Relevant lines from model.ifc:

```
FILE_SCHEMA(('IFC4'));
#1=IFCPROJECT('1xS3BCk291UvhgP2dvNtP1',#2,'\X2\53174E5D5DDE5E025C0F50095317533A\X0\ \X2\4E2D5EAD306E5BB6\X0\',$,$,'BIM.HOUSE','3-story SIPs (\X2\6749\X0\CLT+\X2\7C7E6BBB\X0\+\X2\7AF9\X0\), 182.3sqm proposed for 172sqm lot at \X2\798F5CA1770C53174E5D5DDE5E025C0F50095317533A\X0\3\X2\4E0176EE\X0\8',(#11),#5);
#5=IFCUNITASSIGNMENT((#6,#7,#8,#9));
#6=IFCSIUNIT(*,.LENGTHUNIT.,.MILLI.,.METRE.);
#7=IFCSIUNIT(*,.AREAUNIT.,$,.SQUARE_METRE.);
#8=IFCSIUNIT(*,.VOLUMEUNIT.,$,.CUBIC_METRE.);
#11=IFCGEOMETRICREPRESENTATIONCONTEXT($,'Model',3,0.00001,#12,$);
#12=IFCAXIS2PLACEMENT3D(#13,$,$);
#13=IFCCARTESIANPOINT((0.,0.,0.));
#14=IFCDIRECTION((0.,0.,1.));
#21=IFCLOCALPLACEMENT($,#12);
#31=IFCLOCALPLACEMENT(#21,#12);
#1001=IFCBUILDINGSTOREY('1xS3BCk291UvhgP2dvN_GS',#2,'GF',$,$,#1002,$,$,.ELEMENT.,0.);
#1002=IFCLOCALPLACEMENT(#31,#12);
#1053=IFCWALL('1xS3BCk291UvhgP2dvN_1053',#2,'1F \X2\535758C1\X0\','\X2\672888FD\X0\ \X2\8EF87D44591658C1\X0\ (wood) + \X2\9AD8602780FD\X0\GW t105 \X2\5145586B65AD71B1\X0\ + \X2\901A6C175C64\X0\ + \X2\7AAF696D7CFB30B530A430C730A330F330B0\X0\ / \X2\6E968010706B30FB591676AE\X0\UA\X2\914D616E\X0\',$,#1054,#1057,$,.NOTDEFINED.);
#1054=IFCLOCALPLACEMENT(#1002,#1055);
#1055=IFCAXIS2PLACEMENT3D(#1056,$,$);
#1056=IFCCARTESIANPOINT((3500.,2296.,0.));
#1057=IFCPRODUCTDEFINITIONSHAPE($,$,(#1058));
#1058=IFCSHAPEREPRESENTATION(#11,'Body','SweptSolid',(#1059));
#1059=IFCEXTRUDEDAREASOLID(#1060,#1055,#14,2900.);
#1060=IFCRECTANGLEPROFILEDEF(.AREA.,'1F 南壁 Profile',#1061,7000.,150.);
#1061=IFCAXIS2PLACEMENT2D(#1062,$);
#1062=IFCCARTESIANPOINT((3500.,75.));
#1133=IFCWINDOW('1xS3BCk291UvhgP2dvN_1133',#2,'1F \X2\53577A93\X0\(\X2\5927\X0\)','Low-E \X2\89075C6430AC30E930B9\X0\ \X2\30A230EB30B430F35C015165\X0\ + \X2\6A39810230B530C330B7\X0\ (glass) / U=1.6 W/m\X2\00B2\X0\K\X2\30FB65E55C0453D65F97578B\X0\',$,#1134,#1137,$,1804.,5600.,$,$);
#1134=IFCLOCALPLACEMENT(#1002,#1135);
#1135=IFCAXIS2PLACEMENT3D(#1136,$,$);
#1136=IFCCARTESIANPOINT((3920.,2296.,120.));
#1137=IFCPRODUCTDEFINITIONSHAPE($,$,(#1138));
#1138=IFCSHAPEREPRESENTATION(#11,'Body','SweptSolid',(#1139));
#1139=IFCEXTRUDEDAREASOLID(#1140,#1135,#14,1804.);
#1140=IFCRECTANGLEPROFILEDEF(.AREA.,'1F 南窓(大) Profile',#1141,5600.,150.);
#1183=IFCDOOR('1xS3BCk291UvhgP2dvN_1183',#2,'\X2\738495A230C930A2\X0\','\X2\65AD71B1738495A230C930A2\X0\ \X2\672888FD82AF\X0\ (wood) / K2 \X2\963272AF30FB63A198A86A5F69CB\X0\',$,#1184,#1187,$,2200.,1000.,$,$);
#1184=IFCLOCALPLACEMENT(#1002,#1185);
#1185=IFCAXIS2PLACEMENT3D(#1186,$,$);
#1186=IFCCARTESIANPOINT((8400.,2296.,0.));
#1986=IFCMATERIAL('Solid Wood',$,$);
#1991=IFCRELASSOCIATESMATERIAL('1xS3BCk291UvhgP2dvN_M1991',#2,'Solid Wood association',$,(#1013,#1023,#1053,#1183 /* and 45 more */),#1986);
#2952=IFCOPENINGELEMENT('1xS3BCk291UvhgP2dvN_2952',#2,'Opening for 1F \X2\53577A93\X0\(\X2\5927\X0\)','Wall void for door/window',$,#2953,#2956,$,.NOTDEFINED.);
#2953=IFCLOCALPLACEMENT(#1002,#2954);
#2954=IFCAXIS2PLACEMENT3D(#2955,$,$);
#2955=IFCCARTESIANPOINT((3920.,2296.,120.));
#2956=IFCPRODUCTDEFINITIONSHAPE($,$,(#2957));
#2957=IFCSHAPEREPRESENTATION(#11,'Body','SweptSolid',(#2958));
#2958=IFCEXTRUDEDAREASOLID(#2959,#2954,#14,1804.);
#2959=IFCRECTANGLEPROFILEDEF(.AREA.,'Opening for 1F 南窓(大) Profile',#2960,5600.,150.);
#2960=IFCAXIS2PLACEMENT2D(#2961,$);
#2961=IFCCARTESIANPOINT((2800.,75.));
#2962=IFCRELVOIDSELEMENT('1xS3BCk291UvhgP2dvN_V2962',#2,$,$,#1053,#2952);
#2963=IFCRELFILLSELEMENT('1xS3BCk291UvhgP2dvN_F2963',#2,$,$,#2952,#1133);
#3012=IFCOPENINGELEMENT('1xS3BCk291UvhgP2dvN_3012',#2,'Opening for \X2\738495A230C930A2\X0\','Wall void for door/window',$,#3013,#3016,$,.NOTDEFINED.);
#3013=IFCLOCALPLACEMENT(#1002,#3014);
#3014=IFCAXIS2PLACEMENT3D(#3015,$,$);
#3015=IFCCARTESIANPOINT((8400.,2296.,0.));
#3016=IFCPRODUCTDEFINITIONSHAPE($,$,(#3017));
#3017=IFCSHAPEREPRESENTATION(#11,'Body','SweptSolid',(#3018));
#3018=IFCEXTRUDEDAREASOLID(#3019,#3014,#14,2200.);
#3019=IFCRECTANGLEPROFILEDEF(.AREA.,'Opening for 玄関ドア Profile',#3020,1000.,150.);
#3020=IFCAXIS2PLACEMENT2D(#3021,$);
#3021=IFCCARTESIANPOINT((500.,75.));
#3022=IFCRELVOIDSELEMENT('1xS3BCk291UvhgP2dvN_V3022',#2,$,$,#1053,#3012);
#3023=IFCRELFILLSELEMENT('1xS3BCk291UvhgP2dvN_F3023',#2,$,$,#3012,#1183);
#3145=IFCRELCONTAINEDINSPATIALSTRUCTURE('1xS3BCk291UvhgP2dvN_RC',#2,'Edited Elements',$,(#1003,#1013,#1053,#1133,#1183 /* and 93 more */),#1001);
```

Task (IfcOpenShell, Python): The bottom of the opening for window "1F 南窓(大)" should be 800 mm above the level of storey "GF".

```python
import numpy as np
import ifcopenshell
import ifcopenshell.api.geometry
import ifcopenshell.geom
import ifcopenshell.util.element
import ifcopenshell.util.placement
import ifcopenshell.util.shape
import ifcopenshell.util.unit

model = ifcopenshell.open("model.ifc")
unit_scale = ifcopenshell.util.unit.calculate_unit_scale(model)

window = model.by_guid("1xS3BCk291UvhgP2dvN_1133")
opening = window.FillsVoids[0].RelatingOpeningElement
storey = ifcopenshell.util.element.get_container(window, ifc_class="IfcBuildingStorey")
level = ifcopenshell.util.placement.get_local_placement(storey.ObjectPlacement)[2, 3]

# The opening's origin need not be at the sill, so measure its lowest point.
shape = ifcopenshell.geom.create_shape(ifcopenshell.geom.settings(), opening)
bottom = ifcopenshell.util.shape.get_shape_bottom_elevation(shape, shape.geometry) / unit_scale
dz = level + 0.8 / unit_scale - bottom

shift = np.array([0.0, 0.0, dz])
# The window is not placed relative to its opening, so move both.
for product in (opening, window):
    matrix = ifcopenshell.util.placement.get_local_placement(product.ObjectPlacement)
    matrix[:3, 3] += shift
    ifcopenshell.api.geometry.edit_object_placement(model, product=product, matrix=matrix, is_si=False)

print(f"moved by {dz * unit_scale:+.3f} m")

model.write("model_edited.ifc")
```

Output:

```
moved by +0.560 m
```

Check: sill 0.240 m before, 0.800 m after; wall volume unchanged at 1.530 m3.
